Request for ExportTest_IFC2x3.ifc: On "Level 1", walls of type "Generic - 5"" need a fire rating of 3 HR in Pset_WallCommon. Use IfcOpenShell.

First a look at what the model holds.

```python
import ifcopenshell
import ifcopenshell.util.element

model = ifcopenshell.open("ExportTest_IFC2x3.ifc")
print(model.schema)
storey = next(s for s in model.by_type("IfcBuildingStorey") if s.Name == "Level 1")
walls = [e for e in ifcopenshell.util.element.get_decomposition(storey) if e.is_a("IfcWall")]
seen = {}
for e in walls:
    element_type = ifcopenshell.util.element.get_type(e)
    key = (element_type.Name if element_type != e and element_type else None, ifcopenshell.util.element.get_pset(e, "Pset_WallCommon", "FireRating"))
    seen[key] = seen.get(key, 0) + 1
for (name, value), count in sorted(seen.items(), key=str):
    print(count, "x", name, "|", value)
```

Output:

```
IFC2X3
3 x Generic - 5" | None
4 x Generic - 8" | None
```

```python
import ifcopenshell
import ifcopenshell.api.pset
import ifcopenshell.util.element

model = ifcopenshell.open("ExportTest_IFC2x3.ifc")

storey = next(s for s in model.by_type("IfcBuildingStorey") if s.Name == "Level 1")
walls = [e for e in ifcopenshell.util.element.get_decomposition(storey) if e.is_a("IfcWall")]

count = 0
for e in walls:
    element_type = ifcopenshell.util.element.get_type(e)
    if element_type in (None, e) or element_type.Name != 'Generic - 5"':
        continue
    # add_pset returns the element's existing set when there is one.
    pset = ifcopenshell.api.pset.add_pset(model, product=e, name="Pset_WallCommon")
    ifcopenshell.api.pset.edit_pset(model, pset=pset, properties={"FireRating": "3 HR"})
    count += 1

print(count, "walls updated")

model.write("ExportTest_IFC2x3_v2.ifc")
```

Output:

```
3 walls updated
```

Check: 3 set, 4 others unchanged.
